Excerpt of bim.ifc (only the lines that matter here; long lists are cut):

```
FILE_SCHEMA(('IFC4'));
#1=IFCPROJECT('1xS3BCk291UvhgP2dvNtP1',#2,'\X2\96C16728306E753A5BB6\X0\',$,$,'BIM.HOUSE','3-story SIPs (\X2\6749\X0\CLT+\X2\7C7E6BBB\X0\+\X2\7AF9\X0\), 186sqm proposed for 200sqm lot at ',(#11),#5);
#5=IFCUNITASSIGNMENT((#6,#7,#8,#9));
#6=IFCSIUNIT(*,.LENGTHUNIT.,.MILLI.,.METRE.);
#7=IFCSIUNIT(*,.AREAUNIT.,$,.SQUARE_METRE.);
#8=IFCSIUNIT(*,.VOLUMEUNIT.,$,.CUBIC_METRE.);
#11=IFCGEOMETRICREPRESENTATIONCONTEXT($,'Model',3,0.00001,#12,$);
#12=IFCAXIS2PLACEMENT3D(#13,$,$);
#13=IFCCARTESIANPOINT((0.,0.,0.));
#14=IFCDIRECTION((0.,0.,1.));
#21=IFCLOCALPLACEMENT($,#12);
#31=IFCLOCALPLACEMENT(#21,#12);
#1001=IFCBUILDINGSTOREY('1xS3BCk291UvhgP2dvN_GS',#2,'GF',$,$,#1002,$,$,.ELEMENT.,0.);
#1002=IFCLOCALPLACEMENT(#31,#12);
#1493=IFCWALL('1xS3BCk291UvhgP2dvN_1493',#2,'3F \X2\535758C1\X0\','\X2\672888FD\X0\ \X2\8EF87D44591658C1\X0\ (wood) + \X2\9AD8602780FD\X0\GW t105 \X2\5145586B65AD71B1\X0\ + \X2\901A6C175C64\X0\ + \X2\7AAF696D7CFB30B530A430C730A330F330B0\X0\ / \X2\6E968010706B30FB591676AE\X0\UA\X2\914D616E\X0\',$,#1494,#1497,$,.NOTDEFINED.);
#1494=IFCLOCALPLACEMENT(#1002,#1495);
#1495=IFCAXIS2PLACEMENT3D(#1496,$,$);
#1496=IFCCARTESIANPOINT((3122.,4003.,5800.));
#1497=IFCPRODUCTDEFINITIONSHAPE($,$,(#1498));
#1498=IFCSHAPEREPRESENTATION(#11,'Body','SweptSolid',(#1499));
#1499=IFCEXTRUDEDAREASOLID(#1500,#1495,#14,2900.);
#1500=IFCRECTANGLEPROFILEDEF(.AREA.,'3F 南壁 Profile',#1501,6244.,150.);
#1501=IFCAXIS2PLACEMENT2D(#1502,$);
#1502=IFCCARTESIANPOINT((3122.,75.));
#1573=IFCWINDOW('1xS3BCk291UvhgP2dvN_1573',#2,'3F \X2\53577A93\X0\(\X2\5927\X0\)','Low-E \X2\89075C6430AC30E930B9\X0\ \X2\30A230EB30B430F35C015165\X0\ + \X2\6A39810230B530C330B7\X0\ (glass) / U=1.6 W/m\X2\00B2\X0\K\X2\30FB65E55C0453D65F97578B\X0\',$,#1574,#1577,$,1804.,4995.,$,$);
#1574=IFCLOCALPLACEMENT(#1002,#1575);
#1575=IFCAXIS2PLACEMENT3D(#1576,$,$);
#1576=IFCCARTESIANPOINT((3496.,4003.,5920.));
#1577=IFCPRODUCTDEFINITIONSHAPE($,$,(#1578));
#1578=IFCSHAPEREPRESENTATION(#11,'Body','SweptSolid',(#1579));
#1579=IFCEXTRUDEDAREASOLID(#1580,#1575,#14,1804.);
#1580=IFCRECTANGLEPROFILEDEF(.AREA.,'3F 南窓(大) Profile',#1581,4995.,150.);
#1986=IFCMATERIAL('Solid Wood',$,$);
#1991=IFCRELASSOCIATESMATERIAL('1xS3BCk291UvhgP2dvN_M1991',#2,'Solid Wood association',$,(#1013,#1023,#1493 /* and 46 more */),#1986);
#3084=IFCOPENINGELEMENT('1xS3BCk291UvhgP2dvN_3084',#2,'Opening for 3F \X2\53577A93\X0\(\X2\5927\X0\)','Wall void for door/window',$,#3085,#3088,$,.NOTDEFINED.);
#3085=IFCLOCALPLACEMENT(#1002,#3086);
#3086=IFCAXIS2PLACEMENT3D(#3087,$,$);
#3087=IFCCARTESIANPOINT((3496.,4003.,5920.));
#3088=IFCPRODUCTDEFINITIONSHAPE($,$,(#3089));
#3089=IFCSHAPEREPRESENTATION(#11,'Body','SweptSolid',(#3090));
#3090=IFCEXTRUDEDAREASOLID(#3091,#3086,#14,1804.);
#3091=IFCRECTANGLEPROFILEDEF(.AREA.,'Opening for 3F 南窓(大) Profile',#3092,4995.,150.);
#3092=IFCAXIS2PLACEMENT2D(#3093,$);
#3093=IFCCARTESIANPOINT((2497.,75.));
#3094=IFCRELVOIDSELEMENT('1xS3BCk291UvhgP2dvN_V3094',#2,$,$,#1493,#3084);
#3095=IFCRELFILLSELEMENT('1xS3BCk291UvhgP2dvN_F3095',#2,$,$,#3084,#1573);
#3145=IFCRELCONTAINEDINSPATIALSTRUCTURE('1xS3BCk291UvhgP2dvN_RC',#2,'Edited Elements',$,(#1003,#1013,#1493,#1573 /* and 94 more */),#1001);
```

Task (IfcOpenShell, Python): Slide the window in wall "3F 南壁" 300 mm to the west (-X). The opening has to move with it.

```python
import ifcopenshell
import ifcopenshell.api.geometry
import ifcopenshell.util.placement
import ifcopenshell.util.unit

model = ifcopenshell.open("bim.ifc")
unit_scale = ifcopenshell.util.unit.calculate_unit_scale(model)

window = model.by_guid("1xS3BCk291UvhgP2dvN_1573")
opening = window.FillsVoids[0].RelatingOpeningElement
wall = opening.VoidsElements[0].RelatingBuildingElement

wall_matrix = ifcopenshell.util.placement.get_local_placement(wall.ObjectPlacement)
shift = wall_matrix[:3, 0] * -0.3 / unit_scale
before = ifcopenshell.util.placement.get_local_placement(window.ObjectPlacement)[:3, 3].copy()

# The window is not placed relative to its opening, so move both.
for product in (opening, window):
    matrix = ifcopenshell.util.placement.get_local_placement(product.ObjectPlacement)
    matrix[:3, 3] += shift
    ifcopenshell.api.geometry.edit_object_placement(model, product=product, matrix=matrix, is_si=False)

after = ifcopenshell.util.placement.get_local_placement(window.ObjectPlacement)[:3, 3]
print("window moved by", (after - before).round(3) + 0.0)

model.write("bim_updated.ifc")
```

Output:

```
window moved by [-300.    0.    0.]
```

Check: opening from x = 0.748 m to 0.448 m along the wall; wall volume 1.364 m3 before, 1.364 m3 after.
